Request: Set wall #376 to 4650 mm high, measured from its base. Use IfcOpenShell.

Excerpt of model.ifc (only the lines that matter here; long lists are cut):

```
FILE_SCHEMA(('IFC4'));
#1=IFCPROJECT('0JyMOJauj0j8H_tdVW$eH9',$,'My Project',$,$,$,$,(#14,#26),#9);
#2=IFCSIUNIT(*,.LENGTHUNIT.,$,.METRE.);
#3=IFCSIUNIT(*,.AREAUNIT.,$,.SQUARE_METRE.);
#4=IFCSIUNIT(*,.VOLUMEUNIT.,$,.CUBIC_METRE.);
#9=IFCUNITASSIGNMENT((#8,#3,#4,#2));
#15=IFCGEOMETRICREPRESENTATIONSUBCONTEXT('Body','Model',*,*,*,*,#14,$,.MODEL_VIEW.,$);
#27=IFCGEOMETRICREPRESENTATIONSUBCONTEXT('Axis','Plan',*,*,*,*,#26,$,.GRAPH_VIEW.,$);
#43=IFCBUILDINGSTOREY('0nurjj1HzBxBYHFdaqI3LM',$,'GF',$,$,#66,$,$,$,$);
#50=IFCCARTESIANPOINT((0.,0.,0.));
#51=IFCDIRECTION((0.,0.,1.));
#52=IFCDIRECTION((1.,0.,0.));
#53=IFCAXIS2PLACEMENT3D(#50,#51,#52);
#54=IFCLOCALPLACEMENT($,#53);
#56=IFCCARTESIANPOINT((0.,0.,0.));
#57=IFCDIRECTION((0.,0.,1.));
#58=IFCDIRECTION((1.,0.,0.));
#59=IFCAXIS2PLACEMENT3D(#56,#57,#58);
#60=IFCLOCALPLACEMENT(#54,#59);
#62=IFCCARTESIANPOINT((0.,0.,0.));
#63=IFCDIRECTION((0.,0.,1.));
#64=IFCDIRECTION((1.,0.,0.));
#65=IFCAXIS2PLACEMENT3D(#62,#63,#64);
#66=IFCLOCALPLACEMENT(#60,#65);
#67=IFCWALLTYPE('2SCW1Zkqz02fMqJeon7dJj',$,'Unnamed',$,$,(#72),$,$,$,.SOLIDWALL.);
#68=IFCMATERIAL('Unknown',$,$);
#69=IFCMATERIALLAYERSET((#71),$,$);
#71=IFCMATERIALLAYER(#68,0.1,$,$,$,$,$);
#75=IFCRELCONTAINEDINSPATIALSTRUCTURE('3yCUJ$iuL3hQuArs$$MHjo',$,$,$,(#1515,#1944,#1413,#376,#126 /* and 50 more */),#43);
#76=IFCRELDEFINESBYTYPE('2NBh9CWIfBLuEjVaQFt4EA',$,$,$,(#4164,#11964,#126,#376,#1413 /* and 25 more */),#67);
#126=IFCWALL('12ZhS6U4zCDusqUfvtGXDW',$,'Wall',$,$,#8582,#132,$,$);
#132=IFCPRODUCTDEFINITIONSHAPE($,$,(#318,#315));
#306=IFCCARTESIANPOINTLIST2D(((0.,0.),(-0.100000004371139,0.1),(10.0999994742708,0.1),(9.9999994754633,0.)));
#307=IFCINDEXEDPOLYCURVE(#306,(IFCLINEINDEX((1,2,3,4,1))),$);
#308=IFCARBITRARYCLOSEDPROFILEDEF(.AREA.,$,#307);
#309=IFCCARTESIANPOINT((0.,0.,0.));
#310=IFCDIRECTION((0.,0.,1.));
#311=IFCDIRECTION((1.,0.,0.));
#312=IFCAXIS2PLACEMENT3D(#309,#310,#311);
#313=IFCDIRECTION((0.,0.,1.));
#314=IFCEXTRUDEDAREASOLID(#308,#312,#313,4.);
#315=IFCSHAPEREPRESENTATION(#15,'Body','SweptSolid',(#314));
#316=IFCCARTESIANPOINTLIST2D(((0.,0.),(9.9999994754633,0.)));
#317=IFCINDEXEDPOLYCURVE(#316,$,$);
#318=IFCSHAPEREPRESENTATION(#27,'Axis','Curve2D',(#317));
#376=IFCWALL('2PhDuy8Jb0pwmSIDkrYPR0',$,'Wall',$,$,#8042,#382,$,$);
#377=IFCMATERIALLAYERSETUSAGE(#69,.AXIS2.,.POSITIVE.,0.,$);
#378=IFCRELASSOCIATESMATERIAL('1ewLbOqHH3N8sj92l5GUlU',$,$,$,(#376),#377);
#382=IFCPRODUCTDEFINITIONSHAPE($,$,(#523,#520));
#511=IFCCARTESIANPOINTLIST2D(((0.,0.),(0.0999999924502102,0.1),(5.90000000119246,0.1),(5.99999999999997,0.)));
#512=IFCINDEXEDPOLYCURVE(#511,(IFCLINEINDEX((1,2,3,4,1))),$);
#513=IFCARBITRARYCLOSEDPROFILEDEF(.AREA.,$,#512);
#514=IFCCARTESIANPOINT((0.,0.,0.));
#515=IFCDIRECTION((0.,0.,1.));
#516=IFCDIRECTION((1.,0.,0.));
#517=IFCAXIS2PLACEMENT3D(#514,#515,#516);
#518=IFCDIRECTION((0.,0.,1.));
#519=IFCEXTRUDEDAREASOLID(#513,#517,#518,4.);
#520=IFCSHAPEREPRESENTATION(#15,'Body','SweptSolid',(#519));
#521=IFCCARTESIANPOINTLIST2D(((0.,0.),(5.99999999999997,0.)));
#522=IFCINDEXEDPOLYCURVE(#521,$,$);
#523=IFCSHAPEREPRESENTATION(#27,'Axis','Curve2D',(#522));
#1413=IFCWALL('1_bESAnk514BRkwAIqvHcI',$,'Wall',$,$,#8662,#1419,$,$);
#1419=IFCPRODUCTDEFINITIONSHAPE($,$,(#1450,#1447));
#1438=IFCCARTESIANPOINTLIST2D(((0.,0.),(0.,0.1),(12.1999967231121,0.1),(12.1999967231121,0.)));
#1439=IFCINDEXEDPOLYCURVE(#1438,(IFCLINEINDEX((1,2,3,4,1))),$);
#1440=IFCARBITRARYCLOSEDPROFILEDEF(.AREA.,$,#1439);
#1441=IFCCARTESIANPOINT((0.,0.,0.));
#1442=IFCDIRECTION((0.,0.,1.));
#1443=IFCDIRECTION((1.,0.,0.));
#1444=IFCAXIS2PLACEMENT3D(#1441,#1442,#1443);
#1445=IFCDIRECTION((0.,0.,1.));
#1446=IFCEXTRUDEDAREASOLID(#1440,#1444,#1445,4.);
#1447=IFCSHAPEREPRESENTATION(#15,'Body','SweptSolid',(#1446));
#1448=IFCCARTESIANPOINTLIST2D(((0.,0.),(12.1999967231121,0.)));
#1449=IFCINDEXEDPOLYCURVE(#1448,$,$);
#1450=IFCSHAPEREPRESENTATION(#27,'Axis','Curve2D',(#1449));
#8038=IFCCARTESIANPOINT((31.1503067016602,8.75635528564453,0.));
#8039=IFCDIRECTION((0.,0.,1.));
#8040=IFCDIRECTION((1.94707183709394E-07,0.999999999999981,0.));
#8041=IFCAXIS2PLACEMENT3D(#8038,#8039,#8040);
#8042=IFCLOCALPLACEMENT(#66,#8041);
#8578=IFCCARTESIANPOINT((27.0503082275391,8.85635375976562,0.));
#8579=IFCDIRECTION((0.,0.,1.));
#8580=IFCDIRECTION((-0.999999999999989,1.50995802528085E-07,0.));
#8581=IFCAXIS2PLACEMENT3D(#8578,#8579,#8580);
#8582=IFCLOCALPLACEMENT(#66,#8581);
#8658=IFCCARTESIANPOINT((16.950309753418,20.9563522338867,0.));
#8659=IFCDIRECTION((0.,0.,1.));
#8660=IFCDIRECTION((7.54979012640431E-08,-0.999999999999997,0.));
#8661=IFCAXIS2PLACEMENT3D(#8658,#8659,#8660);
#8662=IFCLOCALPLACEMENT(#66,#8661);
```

```python
import ifcopenshell
import ifcopenshell.geom
import ifcopenshell.util.representation
import ifcopenshell.util.shape
import ifcopenshell.util.unit

model = ifcopenshell.open("model.ifc")
unit_scale = ifcopenshell.util.unit.calculate_unit_scale(model)
settings = ifcopenshell.geom.settings()


def volume(element):
    """Net volume in cubic metres, openings subtracted."""
    shape = ifcopenshell.geom.create_shape(settings, element)
    return ifcopenshell.util.shape.get_volume(shape.geometry)


wall = model.by_id(376)
before = volume(wall)

body = ifcopenshell.util.representation.get_representation(wall, "Model", "Body")
solid = body.Items[0]
old_height = solid.Depth
solid.Depth = 4.65 / unit_scale
after = volume(wall)

print(f"height {old_height:g} -> {solid.Depth:g}, volume {before:.3f} -> {after:.3f} m3")

model.write("model_edited.ifc")
```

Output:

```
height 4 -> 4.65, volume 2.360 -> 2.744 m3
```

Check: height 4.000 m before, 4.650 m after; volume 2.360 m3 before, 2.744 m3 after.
